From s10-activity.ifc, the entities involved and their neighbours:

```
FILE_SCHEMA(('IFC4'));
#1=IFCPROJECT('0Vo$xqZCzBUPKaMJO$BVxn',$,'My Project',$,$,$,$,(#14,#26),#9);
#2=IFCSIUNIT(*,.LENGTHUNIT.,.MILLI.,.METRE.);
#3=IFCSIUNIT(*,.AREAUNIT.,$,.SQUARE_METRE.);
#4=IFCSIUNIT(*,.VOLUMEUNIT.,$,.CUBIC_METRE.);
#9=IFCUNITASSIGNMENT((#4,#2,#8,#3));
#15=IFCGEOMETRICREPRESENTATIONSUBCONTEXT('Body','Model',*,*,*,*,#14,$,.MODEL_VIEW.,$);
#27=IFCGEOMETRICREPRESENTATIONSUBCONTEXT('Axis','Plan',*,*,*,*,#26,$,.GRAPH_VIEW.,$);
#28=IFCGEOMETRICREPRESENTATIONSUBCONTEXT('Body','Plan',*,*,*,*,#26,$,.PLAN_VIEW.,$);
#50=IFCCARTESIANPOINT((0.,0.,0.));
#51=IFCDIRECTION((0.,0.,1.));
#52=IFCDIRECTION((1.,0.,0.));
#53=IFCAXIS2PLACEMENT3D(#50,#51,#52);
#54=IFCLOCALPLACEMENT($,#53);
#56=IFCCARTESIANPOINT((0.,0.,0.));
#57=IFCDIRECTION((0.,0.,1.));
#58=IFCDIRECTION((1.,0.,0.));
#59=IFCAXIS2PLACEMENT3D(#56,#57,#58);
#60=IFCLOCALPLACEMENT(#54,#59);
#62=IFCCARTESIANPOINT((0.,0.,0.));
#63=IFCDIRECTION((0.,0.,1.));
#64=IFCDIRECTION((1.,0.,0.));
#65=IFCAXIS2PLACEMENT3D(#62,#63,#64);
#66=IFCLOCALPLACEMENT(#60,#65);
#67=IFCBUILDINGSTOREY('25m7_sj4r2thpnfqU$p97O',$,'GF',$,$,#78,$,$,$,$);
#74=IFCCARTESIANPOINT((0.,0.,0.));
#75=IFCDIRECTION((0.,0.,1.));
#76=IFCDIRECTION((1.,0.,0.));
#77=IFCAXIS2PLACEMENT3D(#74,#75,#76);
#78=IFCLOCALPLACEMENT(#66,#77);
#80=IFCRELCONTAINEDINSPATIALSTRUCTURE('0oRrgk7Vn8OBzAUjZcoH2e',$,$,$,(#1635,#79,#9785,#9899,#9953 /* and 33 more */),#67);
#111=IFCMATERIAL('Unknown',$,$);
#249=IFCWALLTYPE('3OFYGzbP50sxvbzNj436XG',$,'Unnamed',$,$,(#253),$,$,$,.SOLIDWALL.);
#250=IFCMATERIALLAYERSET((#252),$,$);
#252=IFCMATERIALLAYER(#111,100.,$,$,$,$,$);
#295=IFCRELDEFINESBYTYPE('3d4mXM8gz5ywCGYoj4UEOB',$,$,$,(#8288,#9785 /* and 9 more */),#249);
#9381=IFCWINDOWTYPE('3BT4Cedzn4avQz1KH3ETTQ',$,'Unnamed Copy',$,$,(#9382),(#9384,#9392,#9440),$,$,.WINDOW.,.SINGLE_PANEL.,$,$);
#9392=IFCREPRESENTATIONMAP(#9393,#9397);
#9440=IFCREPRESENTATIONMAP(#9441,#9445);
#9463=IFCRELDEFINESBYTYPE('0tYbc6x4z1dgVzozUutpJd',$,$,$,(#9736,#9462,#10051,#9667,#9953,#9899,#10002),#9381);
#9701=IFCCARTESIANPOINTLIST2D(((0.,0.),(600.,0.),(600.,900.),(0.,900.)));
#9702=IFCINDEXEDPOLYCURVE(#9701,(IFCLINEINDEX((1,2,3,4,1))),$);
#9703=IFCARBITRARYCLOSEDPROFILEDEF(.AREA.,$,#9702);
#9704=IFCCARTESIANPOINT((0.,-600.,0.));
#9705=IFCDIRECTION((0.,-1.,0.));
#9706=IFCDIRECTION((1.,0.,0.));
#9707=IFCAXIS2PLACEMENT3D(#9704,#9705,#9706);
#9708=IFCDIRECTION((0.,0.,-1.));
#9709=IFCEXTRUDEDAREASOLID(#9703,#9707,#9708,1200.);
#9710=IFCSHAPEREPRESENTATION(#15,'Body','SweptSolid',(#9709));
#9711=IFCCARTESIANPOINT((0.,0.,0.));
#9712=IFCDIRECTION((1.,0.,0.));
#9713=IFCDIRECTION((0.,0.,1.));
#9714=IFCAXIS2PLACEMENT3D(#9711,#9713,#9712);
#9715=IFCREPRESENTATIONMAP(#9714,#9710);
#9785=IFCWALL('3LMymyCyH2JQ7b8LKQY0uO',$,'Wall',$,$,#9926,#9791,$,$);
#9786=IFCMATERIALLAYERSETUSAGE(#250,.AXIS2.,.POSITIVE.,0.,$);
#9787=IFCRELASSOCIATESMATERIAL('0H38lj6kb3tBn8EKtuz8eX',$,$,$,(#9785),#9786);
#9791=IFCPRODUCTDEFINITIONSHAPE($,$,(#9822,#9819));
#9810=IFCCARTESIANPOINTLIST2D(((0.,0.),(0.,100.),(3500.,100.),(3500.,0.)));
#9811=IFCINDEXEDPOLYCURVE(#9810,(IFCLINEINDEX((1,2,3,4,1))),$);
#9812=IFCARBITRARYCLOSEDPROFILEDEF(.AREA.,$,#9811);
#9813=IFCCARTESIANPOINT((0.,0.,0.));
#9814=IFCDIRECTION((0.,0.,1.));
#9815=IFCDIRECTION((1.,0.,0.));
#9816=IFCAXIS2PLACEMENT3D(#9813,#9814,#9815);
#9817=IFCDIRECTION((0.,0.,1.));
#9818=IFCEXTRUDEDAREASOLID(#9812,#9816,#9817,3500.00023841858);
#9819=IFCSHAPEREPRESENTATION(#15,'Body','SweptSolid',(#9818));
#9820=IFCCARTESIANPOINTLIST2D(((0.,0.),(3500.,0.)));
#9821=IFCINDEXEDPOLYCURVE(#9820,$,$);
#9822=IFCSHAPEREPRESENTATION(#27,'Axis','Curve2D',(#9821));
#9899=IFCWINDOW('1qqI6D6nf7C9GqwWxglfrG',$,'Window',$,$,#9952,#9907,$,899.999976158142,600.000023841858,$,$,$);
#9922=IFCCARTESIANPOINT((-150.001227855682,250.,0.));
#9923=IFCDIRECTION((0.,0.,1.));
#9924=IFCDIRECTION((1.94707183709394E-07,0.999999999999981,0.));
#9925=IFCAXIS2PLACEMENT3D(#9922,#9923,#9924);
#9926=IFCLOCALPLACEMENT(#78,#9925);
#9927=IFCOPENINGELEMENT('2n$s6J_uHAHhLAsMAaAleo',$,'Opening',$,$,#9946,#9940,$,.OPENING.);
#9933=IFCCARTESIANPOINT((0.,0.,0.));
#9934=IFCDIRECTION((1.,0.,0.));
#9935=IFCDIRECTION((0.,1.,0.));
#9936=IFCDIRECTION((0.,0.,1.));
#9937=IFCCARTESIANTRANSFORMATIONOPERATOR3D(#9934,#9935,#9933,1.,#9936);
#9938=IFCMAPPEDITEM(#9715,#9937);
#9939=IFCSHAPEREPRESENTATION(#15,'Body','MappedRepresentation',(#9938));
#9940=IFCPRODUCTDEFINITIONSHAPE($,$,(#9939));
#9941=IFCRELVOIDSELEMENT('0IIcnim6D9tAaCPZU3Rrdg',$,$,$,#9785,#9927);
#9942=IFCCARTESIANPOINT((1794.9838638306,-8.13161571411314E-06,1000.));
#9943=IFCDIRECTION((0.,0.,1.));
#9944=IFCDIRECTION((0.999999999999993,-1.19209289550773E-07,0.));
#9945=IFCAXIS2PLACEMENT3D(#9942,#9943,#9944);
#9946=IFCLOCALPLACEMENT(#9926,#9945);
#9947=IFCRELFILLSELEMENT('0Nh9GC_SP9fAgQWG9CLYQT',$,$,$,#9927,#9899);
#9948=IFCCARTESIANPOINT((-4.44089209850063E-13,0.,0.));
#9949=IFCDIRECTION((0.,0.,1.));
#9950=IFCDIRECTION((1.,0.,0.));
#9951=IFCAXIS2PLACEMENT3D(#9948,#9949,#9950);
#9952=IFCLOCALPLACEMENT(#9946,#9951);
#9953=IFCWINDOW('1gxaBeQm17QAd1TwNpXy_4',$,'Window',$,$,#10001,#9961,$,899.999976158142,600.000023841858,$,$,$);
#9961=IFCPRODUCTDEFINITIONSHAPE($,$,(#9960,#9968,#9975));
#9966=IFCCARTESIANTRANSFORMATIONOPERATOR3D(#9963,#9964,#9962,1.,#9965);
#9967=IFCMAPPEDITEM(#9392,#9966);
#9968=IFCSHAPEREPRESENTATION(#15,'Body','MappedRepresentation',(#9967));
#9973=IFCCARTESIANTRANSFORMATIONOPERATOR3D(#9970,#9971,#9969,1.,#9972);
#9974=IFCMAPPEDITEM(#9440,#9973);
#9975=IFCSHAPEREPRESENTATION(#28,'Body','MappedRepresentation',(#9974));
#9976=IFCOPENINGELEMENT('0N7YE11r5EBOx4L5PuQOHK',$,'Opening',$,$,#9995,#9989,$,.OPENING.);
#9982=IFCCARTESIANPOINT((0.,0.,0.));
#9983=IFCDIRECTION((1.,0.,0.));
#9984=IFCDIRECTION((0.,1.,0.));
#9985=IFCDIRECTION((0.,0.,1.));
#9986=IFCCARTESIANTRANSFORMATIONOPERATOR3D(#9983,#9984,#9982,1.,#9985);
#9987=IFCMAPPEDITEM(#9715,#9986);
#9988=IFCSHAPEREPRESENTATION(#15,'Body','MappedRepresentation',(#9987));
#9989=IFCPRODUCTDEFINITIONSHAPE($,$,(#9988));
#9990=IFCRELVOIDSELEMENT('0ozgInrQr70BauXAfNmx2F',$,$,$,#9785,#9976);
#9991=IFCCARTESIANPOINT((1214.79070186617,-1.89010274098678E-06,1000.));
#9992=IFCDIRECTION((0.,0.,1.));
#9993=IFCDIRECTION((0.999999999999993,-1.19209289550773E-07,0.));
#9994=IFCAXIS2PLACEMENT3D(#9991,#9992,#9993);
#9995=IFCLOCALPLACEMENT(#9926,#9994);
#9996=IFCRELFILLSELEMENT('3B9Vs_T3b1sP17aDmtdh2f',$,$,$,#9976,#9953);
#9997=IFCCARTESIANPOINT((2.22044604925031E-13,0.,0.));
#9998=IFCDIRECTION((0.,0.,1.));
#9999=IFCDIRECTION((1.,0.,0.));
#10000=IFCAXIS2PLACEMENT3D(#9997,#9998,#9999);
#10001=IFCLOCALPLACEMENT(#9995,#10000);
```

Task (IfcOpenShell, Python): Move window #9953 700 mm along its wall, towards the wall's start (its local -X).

```python
import ifcopenshell
import ifcopenshell.api.geometry
import ifcopenshell.util.placement
import ifcopenshell.util.unit

model = ifcopenshell.open("s10-activity.ifc")
unit_scale = ifcopenshell.util.unit.calculate_unit_scale(model)

window = model.by_guid("1gxaBeQm17QAd1TwNpXy_4")
opening = window.FillsVoids[0].RelatingOpeningElement
wall = opening.VoidsElements[0].RelatingBuildingElement

wall_matrix = ifcopenshell.util.placement.get_local_placement(wall.ObjectPlacement)
shift = wall_matrix[:3, 0] * -0.7 / unit_scale
before = ifcopenshell.util.placement.get_local_placement(window.ObjectPlacement)[:3, 3].copy()

# The window is placed relative to its opening, so it follows when the opening moves.
matrix = ifcopenshell.util.placement.get_local_placement(opening.ObjectPlacement)
matrix[:3, 3] += shift
ifcopenshell.api.geometry.edit_object_placement(
    model, product=opening, matrix=matrix, is_si=False, should_transform_children=True
)

after = ifcopenshell.util.placement.get_local_placement(window.ObjectPlacement)[:3, 3]
print("window moved by", (after - before).round(3) + 0.0)

model.write("s10-activity_updated.ifc")
```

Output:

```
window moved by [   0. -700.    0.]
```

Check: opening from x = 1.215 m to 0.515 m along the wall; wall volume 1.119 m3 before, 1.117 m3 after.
